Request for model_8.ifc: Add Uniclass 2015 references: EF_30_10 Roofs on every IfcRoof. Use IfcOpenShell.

First a look at what the model holds.

```python
import ifcopenshell

model = ifcopenshell.open("model_8.ifc")
print(model.schema)
print("classifications:", [c.Name for c in model.by_type("IfcClassification")])
for ifc_class in ("IfcDoor", "IfcRoof", "IfcStair", "IfcWall", "IfcWindow"):
    print(ifc_class, len(model.by_type(ifc_class)))
```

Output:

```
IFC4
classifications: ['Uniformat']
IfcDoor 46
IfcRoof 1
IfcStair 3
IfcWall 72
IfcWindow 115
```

```python
import ifcopenshell
import ifcopenshell.api.classification

model = ifcopenshell.open("model_8.ifc")

system = ifcopenshell.api.classification.add_classification(model, classification="Uniclass 2015")

codes = {
    "IfcRoof": ("EF_30_10", "Roofs"),
}
for ifc_class, (code, name) in codes.items():
    products = model.by_type(ifc_class)
    ifcopenshell.api.classification.add_reference(
        model, products=products, classification=system, identification=code, name=name
    )
    print(code, len(products))

model.write("model_8_rev.ifc")
```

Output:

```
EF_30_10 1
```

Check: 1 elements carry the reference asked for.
